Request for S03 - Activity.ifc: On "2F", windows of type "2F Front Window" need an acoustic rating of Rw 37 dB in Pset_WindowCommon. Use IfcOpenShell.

First a look at what the model holds.

```python
import ifcopenshell
import ifcopenshell.util.element

model = ifcopenshell.open("S03 - Activity.ifc")
print(model.schema)
storey = next(s for s in model.by_type("IfcBuildingStorey") if s.Name == "2F")
windows = [e for e in ifcopenshell.util.element.get_decomposition(storey) if e.is_a("IfcWindow")]
seen = {}
for e in windows:
    element_type = ifcopenshell.util.element.get_type(e)
    key = (element_type.Name if element_type != e and element_type else None, ifcopenshell.util.element.get_pset(e, "Pset_WindowCommon", "AcousticRating"))
    seen[key] = seen.get(key, 0) + 1
for (name, value), count in sorted(seen.items(), key=str):
    print(count, "x", name, "|", value)
```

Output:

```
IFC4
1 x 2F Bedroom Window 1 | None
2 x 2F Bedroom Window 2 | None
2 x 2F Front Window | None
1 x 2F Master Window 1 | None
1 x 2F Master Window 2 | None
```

```python
import ifcopenshell
import ifcopenshell.api.pset
import ifcopenshell.util.element

model = ifcopenshell.open("S03 - Activity.ifc")

storey = next(s for s in model.by_type("IfcBuildingStorey") if s.Name == "2F")
windows = [e for e in ifcopenshell.util.element.get_decomposition(storey) if e.is_a("IfcWindow")]

count = 0
for e in windows:
    element_type = ifcopenshell.util.element.get_type(e)
    if element_type in (None, e) or element_type.Name != "2F Front Window":
        continue
    # add_pset returns the element's existing set when there is one.
    pset = ifcopenshell.api.pset.add_pset(model, product=e, name="Pset_WindowCommon")
    ifcopenshell.api.pset.edit_pset(model, pset=pset, properties={"AcousticRating": "Rw 37 dB"})
    count += 1

print(count, "windows updated")

model.write("S03 - Activity-out.ifc")
```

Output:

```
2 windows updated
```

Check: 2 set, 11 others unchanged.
